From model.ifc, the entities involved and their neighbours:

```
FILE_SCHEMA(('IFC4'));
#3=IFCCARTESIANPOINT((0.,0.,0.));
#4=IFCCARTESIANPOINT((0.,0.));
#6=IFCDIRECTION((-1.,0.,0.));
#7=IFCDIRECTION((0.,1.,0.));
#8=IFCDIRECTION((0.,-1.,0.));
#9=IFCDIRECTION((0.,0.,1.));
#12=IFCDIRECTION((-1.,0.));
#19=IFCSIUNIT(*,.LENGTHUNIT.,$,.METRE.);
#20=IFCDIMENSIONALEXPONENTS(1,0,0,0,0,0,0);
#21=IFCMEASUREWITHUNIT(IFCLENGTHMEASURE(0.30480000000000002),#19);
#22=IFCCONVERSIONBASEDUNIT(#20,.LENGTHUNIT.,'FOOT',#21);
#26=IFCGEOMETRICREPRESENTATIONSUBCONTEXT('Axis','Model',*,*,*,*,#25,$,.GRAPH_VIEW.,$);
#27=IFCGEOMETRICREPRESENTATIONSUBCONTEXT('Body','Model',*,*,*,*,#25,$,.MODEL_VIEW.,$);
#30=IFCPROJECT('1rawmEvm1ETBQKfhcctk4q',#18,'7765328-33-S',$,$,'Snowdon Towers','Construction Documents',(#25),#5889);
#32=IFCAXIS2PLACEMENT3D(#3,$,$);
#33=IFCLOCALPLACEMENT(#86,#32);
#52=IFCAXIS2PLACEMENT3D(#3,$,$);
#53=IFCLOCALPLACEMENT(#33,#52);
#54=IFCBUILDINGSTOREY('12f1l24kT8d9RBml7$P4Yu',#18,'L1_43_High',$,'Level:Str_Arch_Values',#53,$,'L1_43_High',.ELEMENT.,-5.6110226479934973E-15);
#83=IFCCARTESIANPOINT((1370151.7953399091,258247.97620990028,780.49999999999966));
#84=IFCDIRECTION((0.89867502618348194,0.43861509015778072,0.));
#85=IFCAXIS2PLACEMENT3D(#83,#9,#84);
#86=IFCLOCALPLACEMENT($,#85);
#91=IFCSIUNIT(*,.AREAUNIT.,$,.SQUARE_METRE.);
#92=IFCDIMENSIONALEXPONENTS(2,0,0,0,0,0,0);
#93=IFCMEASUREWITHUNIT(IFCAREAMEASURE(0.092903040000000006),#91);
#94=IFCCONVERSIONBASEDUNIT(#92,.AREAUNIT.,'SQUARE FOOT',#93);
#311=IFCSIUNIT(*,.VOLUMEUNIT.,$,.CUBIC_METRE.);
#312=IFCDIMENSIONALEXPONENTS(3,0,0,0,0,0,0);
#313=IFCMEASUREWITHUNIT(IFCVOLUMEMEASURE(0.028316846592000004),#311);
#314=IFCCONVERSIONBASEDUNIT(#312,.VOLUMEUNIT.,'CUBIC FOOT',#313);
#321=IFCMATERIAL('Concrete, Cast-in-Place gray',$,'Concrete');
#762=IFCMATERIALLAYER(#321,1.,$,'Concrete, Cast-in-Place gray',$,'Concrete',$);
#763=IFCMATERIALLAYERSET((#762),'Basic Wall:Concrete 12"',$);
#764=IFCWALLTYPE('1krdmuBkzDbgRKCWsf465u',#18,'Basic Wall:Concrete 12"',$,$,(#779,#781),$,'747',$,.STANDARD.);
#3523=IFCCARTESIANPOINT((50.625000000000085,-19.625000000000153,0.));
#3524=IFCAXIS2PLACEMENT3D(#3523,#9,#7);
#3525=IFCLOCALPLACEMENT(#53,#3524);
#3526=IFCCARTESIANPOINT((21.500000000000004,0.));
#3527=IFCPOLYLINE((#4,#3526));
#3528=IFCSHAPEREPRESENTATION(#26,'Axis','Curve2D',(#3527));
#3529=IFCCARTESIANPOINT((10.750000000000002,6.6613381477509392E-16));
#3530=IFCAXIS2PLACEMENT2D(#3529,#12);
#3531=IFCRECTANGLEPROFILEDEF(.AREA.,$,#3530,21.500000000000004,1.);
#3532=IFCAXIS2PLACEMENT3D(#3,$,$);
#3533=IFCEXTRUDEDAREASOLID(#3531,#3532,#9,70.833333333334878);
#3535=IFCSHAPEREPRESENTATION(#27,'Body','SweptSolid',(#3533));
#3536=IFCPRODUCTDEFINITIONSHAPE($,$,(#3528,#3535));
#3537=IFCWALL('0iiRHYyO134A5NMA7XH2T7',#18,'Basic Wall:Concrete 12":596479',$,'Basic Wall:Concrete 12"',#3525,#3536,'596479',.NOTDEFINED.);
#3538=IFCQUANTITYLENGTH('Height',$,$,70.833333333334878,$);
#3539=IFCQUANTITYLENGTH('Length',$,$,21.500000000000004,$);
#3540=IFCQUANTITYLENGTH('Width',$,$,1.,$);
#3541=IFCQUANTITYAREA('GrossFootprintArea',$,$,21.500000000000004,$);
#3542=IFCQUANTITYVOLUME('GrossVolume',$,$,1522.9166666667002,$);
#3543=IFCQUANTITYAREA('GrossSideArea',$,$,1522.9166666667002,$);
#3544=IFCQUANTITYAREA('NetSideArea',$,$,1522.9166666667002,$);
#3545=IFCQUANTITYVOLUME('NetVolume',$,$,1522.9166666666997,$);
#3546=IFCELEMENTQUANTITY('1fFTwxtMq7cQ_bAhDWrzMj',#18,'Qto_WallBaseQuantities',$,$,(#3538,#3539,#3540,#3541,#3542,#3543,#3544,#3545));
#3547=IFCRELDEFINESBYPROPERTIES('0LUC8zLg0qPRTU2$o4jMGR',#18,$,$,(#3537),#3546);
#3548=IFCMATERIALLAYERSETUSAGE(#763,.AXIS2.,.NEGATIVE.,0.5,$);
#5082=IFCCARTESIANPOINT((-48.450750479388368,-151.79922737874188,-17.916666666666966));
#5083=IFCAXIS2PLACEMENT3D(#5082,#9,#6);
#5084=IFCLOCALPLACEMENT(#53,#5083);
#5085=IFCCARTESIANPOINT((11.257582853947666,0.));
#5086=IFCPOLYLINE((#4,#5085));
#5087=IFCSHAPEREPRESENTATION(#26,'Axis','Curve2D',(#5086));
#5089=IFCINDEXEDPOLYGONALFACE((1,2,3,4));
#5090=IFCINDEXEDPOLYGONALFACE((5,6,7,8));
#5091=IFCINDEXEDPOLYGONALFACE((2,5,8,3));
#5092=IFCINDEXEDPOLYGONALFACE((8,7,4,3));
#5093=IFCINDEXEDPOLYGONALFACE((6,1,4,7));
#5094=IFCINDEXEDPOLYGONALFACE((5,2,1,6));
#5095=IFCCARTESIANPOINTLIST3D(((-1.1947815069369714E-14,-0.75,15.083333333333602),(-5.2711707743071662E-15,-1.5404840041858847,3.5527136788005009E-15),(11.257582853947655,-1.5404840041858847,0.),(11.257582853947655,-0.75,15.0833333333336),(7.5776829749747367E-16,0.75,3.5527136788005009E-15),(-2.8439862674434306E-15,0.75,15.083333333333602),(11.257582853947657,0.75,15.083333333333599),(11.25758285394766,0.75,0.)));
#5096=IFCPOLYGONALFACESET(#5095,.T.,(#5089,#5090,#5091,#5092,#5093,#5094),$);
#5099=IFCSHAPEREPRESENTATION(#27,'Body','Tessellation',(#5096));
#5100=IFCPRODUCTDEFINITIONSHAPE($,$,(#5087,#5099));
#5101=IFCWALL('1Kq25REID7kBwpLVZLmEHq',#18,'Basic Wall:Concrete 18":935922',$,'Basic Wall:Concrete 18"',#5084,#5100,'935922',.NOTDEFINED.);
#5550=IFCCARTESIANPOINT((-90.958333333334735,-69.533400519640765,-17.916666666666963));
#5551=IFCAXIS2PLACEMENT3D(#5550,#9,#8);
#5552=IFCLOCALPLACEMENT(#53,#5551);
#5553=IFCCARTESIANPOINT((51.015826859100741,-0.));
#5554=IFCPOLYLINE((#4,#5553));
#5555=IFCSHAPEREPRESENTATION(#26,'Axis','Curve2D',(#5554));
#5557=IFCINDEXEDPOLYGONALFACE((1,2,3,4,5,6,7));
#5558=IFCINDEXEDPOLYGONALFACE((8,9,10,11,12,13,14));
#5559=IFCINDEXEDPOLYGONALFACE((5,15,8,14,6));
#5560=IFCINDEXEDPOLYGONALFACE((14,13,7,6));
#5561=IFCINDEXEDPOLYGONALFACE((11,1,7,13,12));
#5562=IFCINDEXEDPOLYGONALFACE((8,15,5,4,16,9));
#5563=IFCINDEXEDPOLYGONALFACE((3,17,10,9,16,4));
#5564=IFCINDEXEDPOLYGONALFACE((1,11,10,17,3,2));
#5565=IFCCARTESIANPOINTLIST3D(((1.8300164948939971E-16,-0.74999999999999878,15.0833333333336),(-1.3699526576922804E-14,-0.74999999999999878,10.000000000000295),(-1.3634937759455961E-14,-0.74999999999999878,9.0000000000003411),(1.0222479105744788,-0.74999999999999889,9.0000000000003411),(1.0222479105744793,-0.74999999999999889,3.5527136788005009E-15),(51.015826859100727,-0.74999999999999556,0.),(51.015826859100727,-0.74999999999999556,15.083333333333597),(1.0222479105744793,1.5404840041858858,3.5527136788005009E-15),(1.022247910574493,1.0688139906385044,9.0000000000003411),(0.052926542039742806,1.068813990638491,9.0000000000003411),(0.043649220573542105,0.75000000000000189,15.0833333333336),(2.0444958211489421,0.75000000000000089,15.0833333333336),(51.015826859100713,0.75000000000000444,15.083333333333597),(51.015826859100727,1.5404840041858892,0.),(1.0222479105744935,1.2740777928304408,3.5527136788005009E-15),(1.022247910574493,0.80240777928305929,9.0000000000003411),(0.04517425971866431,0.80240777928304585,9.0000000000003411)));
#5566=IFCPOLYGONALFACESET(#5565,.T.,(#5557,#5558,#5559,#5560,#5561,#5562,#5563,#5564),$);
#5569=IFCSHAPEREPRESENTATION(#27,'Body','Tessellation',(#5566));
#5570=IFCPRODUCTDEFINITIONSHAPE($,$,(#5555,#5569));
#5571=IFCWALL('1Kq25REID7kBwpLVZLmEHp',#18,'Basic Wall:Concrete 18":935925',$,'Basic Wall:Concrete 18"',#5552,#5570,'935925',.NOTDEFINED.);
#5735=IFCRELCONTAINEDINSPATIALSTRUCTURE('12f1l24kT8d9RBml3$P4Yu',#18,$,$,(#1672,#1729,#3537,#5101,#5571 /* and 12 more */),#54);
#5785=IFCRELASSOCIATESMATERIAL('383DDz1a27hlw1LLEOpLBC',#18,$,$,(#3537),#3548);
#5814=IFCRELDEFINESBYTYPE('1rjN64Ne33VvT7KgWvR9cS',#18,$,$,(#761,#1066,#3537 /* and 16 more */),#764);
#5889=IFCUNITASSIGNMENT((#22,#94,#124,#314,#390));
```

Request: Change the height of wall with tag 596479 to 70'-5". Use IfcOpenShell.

```python
import ifcopenshell
import ifcopenshell.api.pset
import ifcopenshell.geom
import ifcopenshell.util.element
import ifcopenshell.util.representation
import ifcopenshell.util.shape
import ifcopenshell.util.unit

model = ifcopenshell.open("model.ifc")
unit_scale = ifcopenshell.util.unit.calculate_unit_scale(model)
area_scale = ifcopenshell.util.unit.calculate_unit_scale(model, "AREAUNIT")
volume_scale = ifcopenshell.util.unit.calculate_unit_scale(model, "VOLUMEUNIT")
settings = ifcopenshell.geom.settings()


def volume(element):
    """Net volume in cubic metres, openings subtracted."""
    shape = ifcopenshell.geom.create_shape(settings, element)
    return ifcopenshell.util.shape.get_volume(shape.geometry)


wall = model.by_id(3537)
before = volume(wall)

body = ifcopenshell.util.representation.get_representation(wall, "Model", "Body")
solid = body.Items[0]
old_height = solid.Depth
solid.Depth = 845 * 0.0254 / unit_scale
after = volume(wall)
thickness = 0.3048  # wall thickness in metres

# Update the stored height, areas and volumes.
qto = model.by_id(ifcopenshell.util.element.get_pset(wall, "Qto_WallBaseQuantities", should_inherit=False)["id"])
ifcopenshell.api.pset.edit_qto(model, qto=qto, properties={
    "Height": solid.Depth,
    "GrossVolume": ifcopenshell.util.element.get_pset(wall, "Qto_WallBaseQuantities", "GrossVolume") * solid.Depth / old_height,
    "GrossSideArea": ifcopenshell.util.element.get_pset(wall, "Qto_WallBaseQuantities", "GrossSideArea") * solid.Depth / old_height,
    "NetSideArea": after / thickness / area_scale,
    "NetVolume": after / volume_scale,
})

print(f"height {old_height:g} -> {solid.Depth:g}, volume {before:.3f} -> {after:.3f} m3")

model.write("model_rev.ifc")
```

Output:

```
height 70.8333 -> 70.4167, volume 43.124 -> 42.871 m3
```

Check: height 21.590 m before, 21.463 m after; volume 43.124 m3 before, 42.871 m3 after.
